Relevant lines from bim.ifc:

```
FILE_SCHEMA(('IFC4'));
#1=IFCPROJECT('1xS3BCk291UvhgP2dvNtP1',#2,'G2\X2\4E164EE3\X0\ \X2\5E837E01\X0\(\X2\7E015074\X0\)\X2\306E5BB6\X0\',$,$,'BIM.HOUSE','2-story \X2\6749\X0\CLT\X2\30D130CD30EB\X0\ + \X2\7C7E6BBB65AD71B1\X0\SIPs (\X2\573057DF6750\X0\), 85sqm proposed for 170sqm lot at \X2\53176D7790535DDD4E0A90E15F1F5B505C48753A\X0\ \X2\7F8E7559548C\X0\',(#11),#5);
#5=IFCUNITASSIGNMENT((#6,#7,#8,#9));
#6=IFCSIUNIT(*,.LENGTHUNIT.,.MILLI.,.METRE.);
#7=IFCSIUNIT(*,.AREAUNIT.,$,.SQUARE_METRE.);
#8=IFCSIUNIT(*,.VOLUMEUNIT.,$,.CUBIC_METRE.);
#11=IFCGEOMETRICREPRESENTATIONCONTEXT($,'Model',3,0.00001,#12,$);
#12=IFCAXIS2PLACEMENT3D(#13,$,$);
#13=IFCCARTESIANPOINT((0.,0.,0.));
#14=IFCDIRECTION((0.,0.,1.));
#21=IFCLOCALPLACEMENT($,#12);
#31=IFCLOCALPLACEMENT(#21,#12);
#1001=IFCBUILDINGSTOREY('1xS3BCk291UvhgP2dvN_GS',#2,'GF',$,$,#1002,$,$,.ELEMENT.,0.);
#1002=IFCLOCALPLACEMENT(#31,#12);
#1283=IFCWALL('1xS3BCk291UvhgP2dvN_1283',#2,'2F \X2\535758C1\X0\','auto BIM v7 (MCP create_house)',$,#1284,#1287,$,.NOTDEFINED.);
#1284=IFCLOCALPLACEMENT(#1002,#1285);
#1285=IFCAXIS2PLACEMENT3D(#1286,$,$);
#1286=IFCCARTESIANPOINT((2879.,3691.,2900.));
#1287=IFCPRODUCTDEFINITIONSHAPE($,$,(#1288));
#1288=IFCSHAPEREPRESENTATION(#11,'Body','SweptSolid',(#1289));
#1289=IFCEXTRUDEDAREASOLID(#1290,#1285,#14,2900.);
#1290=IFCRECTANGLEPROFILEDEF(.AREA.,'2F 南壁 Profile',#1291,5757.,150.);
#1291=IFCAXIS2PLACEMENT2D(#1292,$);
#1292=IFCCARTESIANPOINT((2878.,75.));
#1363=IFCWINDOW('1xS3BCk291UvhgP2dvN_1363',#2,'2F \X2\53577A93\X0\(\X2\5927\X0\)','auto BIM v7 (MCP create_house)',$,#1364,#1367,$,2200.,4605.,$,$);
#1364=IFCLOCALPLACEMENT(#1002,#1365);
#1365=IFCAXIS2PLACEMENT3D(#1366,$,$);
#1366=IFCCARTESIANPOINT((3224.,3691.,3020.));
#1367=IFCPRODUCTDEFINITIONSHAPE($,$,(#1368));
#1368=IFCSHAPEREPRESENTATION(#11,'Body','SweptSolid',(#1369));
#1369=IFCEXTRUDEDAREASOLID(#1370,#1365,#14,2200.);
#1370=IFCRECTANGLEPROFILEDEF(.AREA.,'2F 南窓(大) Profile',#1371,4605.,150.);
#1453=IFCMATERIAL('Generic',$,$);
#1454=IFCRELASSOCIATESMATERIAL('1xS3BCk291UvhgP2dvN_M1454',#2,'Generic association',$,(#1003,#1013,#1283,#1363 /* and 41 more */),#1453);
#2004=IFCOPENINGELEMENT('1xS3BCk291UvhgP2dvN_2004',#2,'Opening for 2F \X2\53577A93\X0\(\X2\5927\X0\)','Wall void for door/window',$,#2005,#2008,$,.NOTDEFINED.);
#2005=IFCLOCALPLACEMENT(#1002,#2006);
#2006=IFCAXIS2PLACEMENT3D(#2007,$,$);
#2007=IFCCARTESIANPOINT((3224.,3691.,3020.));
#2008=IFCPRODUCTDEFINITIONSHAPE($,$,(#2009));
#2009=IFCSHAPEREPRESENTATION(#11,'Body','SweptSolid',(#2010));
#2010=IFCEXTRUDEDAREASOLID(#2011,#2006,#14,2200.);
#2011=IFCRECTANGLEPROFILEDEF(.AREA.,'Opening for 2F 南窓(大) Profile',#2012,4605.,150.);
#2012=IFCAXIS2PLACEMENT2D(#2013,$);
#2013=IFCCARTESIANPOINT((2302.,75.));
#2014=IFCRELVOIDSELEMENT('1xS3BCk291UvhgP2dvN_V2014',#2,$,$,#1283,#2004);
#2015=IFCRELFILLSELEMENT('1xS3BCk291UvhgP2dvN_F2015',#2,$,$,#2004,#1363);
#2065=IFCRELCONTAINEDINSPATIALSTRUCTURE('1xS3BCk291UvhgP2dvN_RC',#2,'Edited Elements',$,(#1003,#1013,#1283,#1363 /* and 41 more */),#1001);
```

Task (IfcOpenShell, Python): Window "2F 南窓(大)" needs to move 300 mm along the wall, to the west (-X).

```python
import ifcopenshell
import ifcopenshell.api.geometry
import ifcopenshell.util.placement
import ifcopenshell.util.unit

model = ifcopenshell.open("bim.ifc")
unit_scale = ifcopenshell.util.unit.calculate_unit_scale(model)

window = model.by_guid("1xS3BCk291UvhgP2dvN_1363")
opening = window.FillsVoids[0].RelatingOpeningElement
wall = opening.VoidsElements[0].RelatingBuildingElement

wall_matrix = ifcopenshell.util.placement.get_local_placement(wall.ObjectPlacement)
shift = wall_matrix[:3, 0] * -0.3 / unit_scale
before = ifcopenshell.util.placement.get_local_placement(window.ObjectPlacement)[:3, 3].copy()

# The window is not placed relative to its opening, so move both.
for product in (opening, window):
    matrix = ifcopenshell.util.placement.get_local_placement(product.ObjectPlacement)
    matrix[:3, 3] += shift
    ifcopenshell.api.geometry.edit_object_placement(model, product=product, matrix=matrix, is_si=False)

after = ifcopenshell.util.placement.get_local_placement(window.ObjectPlacement)[:3, 3]
print("window moved by", (after - before).round(3) + 0.0)

model.write("bim_rev.ifc")
```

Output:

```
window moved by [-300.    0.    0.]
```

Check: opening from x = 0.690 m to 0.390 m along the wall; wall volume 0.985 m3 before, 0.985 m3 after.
